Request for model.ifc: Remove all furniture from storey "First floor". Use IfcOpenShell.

First a look at what the model holds.

```python
import ifcopenshell
import ifcopenshell.util.element

model = ifcopenshell.open("model.ifc")
print(model.schema)
storey = next(s for s in model.by_type("IfcBuildingStorey") if s.Name == "First floor")
furniture = [e for e in ifcopenshell.util.element.get_decomposition(storey) if e.is_a("IfcFurnishingElement")]
seen = {}
for e in furniture:
    element_type = ifcopenshell.util.element.get_type(e)
    name = element_type.Name if element_type not in (None, e) else None
    seen[name] = seen.get(name, 0) + 1
for name, count in sorted(seen.items(), key=str):
    print(count, "x", name)
```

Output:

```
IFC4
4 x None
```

```python
import ifcopenshell
import ifcopenshell.api.root
import ifcopenshell.util.element

model = ifcopenshell.open("model.ifc")

storey = next(s for s in model.by_type("IfcBuildingStorey") if s.Name == "First floor")
furniture = [e for e in ifcopenshell.util.element.get_decomposition(storey) if e.is_a("IfcFurnishingElement")]

for e in furniture:
    ifcopenshell.api.root.remove_product(model, product=e)
print(len(furniture), "removed")

model.write("model-out.ifc")
```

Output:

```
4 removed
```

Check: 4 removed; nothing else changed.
